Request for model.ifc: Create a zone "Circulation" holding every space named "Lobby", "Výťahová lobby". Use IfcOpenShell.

First a look at what the model holds.

```python
import ifcopenshell

model = ifcopenshell.open("model.ifc")
print(model.schema)
seen = {}
for space in model.by_type("IfcSpace"):
    seen[space.LongName] = seen.get(space.LongName, 0) + 1
for name, count in sorted(seen.items(), key=str):
    print(count, "x", name)
print("zones:", [z.Name for z in model.by_type("IfcZone")][:20])
```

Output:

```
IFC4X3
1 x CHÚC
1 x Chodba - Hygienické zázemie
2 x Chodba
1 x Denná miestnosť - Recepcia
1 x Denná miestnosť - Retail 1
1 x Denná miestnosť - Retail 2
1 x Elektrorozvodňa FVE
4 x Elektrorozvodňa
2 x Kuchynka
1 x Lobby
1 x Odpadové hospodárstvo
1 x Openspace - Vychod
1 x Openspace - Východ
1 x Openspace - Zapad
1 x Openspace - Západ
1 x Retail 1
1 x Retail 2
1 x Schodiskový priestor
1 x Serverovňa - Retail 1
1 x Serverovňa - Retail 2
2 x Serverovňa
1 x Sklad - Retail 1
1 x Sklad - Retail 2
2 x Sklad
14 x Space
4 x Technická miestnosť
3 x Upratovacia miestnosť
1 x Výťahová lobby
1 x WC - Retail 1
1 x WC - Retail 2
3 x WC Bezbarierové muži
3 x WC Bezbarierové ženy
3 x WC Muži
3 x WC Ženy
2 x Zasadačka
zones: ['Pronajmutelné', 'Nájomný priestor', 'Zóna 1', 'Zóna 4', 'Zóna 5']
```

```python
import ifcopenshell
import ifcopenshell.api.group
import ifcopenshell.api.root

model = ifcopenshell.open("model.ifc")

names = {"Lobby", "Výťahová lobby"}
spaces = [s for s in model.by_type("IfcSpace") if s.LongName in names]

zone = ifcopenshell.api.root.create_entity(model, ifc_class="IfcZone", name="Circulation")
ifcopenshell.api.group.assign_group(model, products=spaces, group=zone)
print(len(spaces), "spaces in", zone.Name)

model.write("model-out.ifc")
```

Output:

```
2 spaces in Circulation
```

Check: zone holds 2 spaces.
